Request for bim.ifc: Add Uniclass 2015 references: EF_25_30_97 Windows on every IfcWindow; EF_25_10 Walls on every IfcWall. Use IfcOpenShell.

First a look at what the model holds.

```python
import ifcopenshell

model = ifcopenshell.open("bim.ifc")
print(model.schema)
print("classifications:", [c.Name for c in model.by_type("IfcClassification")])
for ifc_class in ("IfcDoor", "IfcRoof", "IfcStair", "IfcWall", "IfcWindow"):
    print(ifc_class, len(model.by_type(ifc_class)))
```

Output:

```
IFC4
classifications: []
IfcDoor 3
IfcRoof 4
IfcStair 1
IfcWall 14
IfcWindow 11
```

```python
import ifcopenshell
import ifcopenshell.api.classification

model = ifcopenshell.open("bim.ifc")

system = ifcopenshell.api.classification.add_classification(model, classification="Uniclass 2015")

codes = {
    "IfcWindow": ("EF_25_30_97", "Windows"),
    "IfcWall": ("EF_25_10", "Walls"),
}
for ifc_class, (code, name) in codes.items():
    products = model.by_type(ifc_class)
    ifcopenshell.api.classification.add_reference(
        model, products=products, classification=system, identification=code, name=name
    )
    print(code, len(products))

model.write("bim_v2.ifc")
```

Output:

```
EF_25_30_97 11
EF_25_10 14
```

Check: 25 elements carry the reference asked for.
